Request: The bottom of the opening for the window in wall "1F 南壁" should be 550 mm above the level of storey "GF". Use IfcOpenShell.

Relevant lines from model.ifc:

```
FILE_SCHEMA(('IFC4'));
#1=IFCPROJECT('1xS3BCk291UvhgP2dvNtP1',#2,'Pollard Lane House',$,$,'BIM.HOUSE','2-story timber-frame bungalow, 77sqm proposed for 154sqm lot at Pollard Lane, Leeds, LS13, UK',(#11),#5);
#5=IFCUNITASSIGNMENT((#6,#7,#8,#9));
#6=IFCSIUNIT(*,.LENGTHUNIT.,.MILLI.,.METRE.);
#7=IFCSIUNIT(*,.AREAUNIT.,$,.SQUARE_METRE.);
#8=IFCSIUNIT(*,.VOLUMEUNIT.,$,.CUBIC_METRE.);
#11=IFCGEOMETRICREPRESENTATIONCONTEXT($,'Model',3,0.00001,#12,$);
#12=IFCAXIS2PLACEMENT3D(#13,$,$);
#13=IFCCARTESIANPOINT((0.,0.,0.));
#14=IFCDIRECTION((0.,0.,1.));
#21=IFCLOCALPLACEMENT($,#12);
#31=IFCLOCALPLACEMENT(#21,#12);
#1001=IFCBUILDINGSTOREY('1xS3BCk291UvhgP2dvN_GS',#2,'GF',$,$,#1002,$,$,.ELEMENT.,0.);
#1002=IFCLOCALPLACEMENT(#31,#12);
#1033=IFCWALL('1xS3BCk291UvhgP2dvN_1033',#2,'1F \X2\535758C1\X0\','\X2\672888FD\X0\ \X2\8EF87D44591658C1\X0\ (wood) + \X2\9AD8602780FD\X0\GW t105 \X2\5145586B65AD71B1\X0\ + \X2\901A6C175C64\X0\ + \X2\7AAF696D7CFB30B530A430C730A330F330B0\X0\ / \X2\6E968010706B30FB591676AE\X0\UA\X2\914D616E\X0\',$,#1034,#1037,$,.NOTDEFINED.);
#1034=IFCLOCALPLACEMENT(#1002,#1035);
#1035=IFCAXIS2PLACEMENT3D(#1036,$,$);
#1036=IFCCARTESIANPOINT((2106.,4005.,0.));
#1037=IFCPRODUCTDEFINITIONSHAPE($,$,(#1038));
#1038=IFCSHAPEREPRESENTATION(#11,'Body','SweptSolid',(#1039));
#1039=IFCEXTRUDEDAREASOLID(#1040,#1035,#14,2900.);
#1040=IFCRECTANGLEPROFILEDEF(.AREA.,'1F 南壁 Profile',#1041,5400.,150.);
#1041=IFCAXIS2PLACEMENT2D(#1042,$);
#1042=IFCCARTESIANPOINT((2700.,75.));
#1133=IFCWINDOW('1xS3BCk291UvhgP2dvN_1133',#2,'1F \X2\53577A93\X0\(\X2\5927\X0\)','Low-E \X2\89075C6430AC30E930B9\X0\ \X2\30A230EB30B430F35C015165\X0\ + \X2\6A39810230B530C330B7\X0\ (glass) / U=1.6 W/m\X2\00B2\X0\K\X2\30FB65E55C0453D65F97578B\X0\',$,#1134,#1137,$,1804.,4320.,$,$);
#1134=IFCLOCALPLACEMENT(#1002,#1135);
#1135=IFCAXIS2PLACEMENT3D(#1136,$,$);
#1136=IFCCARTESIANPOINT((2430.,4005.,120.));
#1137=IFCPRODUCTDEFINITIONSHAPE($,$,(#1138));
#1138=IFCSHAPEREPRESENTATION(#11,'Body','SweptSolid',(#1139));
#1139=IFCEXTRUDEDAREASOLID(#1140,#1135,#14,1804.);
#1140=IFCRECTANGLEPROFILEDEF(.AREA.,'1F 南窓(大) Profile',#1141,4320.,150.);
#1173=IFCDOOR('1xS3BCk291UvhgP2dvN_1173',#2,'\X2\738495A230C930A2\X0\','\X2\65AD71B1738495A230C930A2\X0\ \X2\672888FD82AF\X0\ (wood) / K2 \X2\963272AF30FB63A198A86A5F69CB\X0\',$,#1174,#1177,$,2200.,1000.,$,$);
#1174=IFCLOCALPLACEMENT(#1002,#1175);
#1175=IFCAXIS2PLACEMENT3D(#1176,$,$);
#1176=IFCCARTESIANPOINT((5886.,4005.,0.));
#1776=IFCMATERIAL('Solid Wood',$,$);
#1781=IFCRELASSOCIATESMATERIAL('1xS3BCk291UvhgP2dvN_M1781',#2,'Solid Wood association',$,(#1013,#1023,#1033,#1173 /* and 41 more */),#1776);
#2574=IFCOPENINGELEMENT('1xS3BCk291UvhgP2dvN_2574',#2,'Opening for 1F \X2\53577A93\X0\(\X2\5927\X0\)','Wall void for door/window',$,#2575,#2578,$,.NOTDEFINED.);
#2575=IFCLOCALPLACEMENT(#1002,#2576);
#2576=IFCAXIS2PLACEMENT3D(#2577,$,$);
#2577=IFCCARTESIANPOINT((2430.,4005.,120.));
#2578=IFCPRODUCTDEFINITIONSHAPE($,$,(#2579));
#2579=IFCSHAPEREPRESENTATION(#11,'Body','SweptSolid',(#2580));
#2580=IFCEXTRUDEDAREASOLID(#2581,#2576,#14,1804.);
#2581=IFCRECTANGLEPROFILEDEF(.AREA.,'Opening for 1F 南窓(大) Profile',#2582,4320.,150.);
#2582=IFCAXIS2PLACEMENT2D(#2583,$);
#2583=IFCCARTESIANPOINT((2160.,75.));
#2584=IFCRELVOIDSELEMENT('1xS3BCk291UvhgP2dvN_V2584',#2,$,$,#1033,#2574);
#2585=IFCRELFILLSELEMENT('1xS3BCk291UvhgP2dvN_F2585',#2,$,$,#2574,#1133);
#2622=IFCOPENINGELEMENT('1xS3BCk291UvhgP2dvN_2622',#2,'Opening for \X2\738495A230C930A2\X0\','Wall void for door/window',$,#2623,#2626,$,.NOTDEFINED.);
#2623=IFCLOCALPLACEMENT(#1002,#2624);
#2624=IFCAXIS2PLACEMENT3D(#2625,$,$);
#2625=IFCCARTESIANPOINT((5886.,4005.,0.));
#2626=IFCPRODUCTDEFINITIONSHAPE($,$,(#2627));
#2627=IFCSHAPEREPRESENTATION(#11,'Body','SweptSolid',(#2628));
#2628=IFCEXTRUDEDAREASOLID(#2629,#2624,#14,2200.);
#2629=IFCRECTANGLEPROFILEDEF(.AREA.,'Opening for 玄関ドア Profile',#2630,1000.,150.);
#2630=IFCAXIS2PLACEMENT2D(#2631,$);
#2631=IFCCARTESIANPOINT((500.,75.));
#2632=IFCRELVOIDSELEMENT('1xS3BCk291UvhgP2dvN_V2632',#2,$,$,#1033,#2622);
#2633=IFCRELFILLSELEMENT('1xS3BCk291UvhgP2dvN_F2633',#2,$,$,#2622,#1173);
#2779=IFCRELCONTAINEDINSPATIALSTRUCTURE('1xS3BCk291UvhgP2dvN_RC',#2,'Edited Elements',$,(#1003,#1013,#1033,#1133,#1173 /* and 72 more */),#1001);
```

```python
import numpy as np
import ifcopenshell
import ifcopenshell.api.geometry
import ifcopenshell.geom
import ifcopenshell.util.element
import ifcopenshell.util.placement
import ifcopenshell.util.shape
import ifcopenshell.util.unit

model = ifcopenshell.open("model.ifc")
unit_scale = ifcopenshell.util.unit.calculate_unit_scale(model)

window = model.by_guid("1xS3BCk291UvhgP2dvN_1133")
opening = window.FillsVoids[0].RelatingOpeningElement
storey = ifcopenshell.util.element.get_container(window, ifc_class="IfcBuildingStorey")
level = ifcopenshell.util.placement.get_local_placement(storey.ObjectPlacement)[2, 3]

# The opening's origin need not be at the sill, so measure its lowest point.
shape = ifcopenshell.geom.create_shape(ifcopenshell.geom.settings(), opening)
bottom = ifcopenshell.util.shape.get_shape_bottom_elevation(shape, shape.geometry) / unit_scale
dz = level + 550.0 - bottom

shift = np.array([0.0, 0.0, dz])
# The window is not placed relative to its opening, so move both.
for product in (opening, window):
    matrix = ifcopenshell.util.placement.get_local_placement(product.ObjectPlacement)
    matrix[:3, 3] += shift
    ifcopenshell.api.geometry.edit_object_placement(model, product=product, matrix=matrix, is_si=False)

print(f"moved by {dz * unit_scale:+.3f} m")

model.write("model_v2.ifc")
```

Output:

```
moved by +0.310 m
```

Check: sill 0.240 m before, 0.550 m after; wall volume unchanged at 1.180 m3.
